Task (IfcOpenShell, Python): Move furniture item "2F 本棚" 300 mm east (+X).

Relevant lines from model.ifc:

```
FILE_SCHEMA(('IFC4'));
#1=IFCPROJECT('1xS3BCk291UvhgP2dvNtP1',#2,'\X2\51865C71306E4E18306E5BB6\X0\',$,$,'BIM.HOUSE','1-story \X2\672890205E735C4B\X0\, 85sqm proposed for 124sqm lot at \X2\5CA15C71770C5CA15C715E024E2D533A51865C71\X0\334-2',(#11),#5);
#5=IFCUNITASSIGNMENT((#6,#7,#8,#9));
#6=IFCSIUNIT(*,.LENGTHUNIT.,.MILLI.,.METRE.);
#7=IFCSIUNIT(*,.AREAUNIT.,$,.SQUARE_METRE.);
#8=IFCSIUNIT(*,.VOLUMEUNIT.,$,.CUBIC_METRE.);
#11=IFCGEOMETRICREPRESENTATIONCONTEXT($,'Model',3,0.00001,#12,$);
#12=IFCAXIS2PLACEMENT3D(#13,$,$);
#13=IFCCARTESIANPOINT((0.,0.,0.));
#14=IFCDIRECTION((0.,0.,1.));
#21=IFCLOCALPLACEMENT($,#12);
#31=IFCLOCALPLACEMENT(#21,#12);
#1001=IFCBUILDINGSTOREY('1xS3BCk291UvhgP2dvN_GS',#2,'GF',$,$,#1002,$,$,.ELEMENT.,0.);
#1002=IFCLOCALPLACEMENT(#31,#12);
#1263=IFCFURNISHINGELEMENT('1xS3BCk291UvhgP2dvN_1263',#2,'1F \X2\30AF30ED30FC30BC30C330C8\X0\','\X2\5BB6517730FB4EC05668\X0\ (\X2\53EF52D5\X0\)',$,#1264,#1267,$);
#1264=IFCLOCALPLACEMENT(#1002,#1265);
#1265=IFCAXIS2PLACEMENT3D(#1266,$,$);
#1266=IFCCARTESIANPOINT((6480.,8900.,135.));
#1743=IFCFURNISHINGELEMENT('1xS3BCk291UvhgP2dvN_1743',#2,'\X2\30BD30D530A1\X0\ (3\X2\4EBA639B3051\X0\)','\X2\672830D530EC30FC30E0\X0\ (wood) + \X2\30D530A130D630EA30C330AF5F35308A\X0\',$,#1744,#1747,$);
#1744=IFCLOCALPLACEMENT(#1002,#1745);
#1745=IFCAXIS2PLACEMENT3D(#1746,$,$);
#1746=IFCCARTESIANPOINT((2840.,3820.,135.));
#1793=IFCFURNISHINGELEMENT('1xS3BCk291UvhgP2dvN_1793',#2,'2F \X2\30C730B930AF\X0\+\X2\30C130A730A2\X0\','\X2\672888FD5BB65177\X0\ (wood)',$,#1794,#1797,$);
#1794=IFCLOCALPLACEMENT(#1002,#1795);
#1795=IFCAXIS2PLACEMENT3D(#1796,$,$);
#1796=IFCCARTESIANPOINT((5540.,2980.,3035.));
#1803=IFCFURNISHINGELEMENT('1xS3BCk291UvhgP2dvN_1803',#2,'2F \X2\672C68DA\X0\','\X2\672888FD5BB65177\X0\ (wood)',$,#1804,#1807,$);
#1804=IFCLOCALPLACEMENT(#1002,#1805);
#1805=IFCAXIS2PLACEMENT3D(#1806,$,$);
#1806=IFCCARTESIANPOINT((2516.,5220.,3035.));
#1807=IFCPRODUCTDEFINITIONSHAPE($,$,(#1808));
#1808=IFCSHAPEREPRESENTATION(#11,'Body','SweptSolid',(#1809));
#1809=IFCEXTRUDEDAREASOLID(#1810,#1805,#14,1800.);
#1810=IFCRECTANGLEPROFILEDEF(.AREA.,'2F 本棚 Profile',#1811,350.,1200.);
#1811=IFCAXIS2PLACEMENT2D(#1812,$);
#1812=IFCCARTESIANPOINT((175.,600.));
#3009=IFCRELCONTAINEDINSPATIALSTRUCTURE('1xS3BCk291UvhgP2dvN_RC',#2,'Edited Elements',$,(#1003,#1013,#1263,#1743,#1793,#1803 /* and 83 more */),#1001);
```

```python
import ifcopenshell
import ifcopenshell.api.geometry
import ifcopenshell.util.placement
import ifcopenshell.util.unit

model = ifcopenshell.open("model.ifc")
unit_scale = ifcopenshell.util.unit.calculate_unit_scale(model)

item = model.by_guid("1xS3BCk291UvhgP2dvN_1803")
matrix = ifcopenshell.util.placement.get_local_placement(item.ObjectPlacement)
matrix[0, 3] += 0.3 / unit_scale
ifcopenshell.api.geometry.edit_object_placement(model, product=item, matrix=matrix, is_si=False)

print(ifcopenshell.util.placement.get_local_placement(item.ObjectPlacement).round(3) + 0.0)

model.write("model_updated.ifc")
```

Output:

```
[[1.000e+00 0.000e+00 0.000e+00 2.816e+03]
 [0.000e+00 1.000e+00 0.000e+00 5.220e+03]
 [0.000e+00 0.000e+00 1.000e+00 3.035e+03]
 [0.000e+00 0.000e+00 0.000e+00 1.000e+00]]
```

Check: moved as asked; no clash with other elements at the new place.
